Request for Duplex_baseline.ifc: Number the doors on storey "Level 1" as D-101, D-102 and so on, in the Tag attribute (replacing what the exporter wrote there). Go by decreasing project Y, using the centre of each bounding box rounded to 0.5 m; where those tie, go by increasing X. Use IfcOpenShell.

First a look at what the model holds.

```python
import ifcopenshell
import ifcopenshell.util.element
import ifcopenshell.util.placement

model = ifcopenshell.open("Duplex_baseline.ifc")
print(model.schema)
storey = next(s for s in model.by_type("IfcBuildingStorey") if s.Name == "Level 1")
doors = [e for e in ifcopenshell.util.element.get_decomposition(storey) if e.is_a("IfcDoor")]
for e in sorted(doors, key=lambda e: e.id()):
    origin = ifcopenshell.util.placement.get_local_placement(e.ObjectPlacement)[:3, 3]
    print(e.id(), e.Tag, e.Name, origin.round(2) + 0.0, sep=" | ")
```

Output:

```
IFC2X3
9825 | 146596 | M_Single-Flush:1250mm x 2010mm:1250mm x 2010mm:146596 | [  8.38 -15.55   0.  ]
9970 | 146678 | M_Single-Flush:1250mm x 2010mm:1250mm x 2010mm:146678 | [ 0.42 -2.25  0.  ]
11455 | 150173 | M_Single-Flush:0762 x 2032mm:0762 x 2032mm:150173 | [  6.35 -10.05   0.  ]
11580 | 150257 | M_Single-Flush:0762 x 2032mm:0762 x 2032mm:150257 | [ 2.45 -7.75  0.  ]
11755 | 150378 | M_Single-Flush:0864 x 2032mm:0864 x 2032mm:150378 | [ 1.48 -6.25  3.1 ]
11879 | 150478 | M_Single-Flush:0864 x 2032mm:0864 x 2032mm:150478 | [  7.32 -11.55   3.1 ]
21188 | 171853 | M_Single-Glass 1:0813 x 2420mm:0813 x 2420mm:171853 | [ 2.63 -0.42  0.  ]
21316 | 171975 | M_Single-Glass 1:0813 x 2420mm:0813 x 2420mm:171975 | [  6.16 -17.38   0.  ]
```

```python
import ifcopenshell
import ifcopenshell.geom
import ifcopenshell.util.element
import ifcopenshell.util.shape

model = ifcopenshell.open("Duplex_baseline.ifc")
settings = ifcopenshell.geom.settings()
settings.set("use-world-coords", True)


def centre(element):
    shape = ifcopenshell.geom.create_shape(settings, element)
    return ifcopenshell.util.shape.get_bbox_centroid(shape.geometry)


storey = next(s for s in model.by_type("IfcBuildingStorey") if s.Name == "Level 1")
doors = [e for e in ifcopenshell.util.element.get_decomposition(storey) if e.is_a("IfcDoor")]

# Insertion points can sit at a corner or the storey origin, so sort by the geometry (in metres).
centres = {e: centre(e) for e in doors}
doors.sort(key=lambda e: (-round(centres[e][1] / 0.5), centres[e][0]))

for i, e in enumerate(doors, start=1):
    number = f"D-1{i:02d}"
    e.Tag = number
    print(e.id(), number)

model.write("Duplex_baseline-out.ifc")
```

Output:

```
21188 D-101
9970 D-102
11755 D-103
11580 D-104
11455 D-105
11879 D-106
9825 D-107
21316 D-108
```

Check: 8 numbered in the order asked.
